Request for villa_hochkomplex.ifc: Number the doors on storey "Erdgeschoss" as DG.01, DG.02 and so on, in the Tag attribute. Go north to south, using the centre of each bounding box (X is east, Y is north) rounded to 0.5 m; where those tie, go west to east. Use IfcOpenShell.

First a look at what the model holds.

```python
import ifcopenshell
import ifcopenshell.util.element
import ifcopenshell.util.placement

model = ifcopenshell.open("villa_hochkomplex.ifc")
print(model.schema)
storey = next(s for s in model.by_type("IfcBuildingStorey") if s.Name == "Erdgeschoss")
doors = [e for e in ifcopenshell.util.element.get_decomposition(storey) if e.is_a("IfcDoor")]
for e in sorted(doors, key=lambda e: e.id()):
    origin = ifcopenshell.util.placement.get_local_placement(e.ObjectPlacement)[:3, 3]
    print(e.id(), e.Tag, e.Name, origin.round(2) + 0.0, sep=" | ")
```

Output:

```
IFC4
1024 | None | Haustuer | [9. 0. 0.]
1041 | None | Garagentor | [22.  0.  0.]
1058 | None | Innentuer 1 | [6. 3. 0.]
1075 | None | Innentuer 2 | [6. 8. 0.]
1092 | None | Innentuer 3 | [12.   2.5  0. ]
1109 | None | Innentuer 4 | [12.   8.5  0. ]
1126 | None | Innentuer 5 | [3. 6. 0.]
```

```python
import ifcopenshell
import ifcopenshell.geom
import ifcopenshell.util.element
import ifcopenshell.util.shape

model = ifcopenshell.open("villa_hochkomplex.ifc")
settings = ifcopenshell.geom.settings()
settings.set("use-world-coords", True)


def centre(element):
    shape = ifcopenshell.geom.create_shape(settings, element)
    return ifcopenshell.util.shape.get_bbox_centroid(shape.geometry)


storey = next(s for s in model.by_type("IfcBuildingStorey") if s.Name == "Erdgeschoss")
doors = [e for e in ifcopenshell.util.element.get_decomposition(storey) if e.is_a("IfcDoor")]

# Insertion points can sit at a corner or the storey origin, so sort by the geometry (in metres).
centres = {e: centre(e) for e in doors}
doors.sort(key=lambda e: (-round(centres[e][1] / 0.5), centres[e][0]))

for i, e in enumerate(doors, start=1):
    number = f"DG.{i:02d}"
    e.Tag = number
    print(e.id(), number)

model.write("villa_hochkomplex_v2.ifc")
```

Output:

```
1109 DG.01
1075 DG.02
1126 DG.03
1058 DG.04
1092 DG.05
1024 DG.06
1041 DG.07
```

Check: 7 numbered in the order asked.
